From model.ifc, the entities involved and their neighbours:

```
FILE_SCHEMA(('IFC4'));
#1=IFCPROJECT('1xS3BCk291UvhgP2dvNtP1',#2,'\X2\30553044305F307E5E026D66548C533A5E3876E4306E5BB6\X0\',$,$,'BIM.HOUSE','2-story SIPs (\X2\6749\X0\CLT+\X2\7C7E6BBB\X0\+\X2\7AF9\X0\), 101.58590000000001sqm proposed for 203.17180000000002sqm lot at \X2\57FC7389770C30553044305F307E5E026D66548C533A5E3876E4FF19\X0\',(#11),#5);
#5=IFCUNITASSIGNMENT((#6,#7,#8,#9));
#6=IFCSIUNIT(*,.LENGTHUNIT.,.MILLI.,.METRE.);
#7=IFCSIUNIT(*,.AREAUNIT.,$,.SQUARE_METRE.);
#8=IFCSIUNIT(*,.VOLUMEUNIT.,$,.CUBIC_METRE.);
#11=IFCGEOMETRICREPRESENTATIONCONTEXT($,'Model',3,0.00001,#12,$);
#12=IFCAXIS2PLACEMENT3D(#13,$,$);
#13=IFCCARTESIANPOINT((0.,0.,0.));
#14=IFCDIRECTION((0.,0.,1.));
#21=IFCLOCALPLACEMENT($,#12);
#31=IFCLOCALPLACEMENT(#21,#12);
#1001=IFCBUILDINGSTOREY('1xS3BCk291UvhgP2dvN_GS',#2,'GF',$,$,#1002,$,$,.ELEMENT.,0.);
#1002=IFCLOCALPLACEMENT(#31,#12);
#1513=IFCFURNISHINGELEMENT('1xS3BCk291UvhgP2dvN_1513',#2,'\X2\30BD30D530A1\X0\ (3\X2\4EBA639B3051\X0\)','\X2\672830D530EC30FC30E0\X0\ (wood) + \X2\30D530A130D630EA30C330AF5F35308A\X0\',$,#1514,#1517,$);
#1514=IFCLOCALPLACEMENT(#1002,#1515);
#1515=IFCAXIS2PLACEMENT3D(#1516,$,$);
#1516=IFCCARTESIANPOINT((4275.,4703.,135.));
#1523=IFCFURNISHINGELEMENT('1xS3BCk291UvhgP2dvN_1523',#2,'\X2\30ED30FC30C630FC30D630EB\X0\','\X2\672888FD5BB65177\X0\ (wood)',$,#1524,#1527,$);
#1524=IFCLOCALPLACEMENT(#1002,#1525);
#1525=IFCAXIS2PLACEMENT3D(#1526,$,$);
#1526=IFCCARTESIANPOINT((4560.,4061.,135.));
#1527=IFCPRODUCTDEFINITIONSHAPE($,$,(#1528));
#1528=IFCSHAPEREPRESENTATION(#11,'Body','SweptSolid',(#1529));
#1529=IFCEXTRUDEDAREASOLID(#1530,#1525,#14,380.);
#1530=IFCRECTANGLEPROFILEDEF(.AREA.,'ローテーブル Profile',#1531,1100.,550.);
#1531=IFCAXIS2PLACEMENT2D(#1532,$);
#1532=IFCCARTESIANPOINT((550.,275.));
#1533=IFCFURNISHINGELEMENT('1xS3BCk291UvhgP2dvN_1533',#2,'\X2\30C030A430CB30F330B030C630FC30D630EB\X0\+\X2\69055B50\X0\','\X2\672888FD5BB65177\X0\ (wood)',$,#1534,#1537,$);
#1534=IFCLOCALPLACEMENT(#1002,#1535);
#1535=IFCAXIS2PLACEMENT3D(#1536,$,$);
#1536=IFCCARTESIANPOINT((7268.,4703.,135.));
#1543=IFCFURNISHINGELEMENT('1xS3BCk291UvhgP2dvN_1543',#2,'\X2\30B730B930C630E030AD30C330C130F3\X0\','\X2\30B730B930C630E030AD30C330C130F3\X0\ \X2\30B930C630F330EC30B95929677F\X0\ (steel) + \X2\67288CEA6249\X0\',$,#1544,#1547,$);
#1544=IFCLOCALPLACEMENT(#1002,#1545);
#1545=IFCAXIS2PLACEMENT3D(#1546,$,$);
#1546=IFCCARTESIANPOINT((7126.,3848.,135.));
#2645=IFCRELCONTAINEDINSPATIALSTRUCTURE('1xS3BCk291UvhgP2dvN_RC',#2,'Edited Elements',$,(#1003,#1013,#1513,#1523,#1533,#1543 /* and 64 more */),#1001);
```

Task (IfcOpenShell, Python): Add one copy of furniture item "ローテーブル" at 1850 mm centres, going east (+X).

```python
import numpy as np
import ifcopenshell
import ifcopenshell.api.geometry
import ifcopenshell.api.root
import ifcopenshell.util.element
import ifcopenshell.util.placement
import ifcopenshell.util.unit

model = ifcopenshell.open("model.ifc")
unit_scale = ifcopenshell.util.unit.calculate_unit_scale(model)


def reuse_history(source, copy):
    """copy_class also copies each property set's owner history, people and application; keep the originals."""
    for rel in copy.IsDefinedBy:
        if rel.is_a("IfcRelDefinesByProperties") and (history := rel.RelatingPropertyDefinition.OwnerHistory):
            rel.RelatingPropertyDefinition.OwnerHistory = source.OwnerHistory
            ifcopenshell.util.element.remove_deep2(model, history)


source = model.by_guid("1xS3BCk291UvhgP2dvN_1523")
base = ifcopenshell.util.placement.get_local_placement(source.ObjectPlacement)
step = np.array([1.0, 0.0, 0.0]) * 1.85 / unit_scale

for i in range(1, 2):
    copy = ifcopenshell.api.root.copy_class(model, product=source)
    copy.Representation = ifcopenshell.util.element.copy_deep(
        model, source.Representation, exclude=["IfcGeometricRepresentationContext", "IfcRepresentationMap"]
    )
    reuse_history(source, copy)
    matrix = base.copy()
    matrix[:3, 3] += i * step
    print("added at", matrix[:3, 3].round(3) + 0.0)
    ifcopenshell.api.geometry.edit_object_placement(model, product=copy, matrix=matrix, is_si=False)

model.write("model_v2.ifc")
```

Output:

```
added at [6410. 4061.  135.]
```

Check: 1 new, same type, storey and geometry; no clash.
